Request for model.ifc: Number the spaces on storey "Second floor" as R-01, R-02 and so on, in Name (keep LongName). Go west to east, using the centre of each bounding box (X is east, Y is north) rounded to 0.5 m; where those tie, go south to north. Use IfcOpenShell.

First a look at what the model holds.

```python
import ifcopenshell
import ifcopenshell.util.element
import ifcopenshell.util.placement

model = ifcopenshell.open("model.ifc")
print(model.schema)
storey = next(s for s in model.by_type("IfcBuildingStorey") if s.Name == "Second floor")
spaces = [e for e in ifcopenshell.util.element.get_decomposition(storey) if e.is_a("IfcSpace")]
for e in sorted(spaces, key=lambda e: e.id()):
    origin = ifcopenshell.util.placement.get_local_placement(e.ObjectPlacement)[:3, 3]
    print(e.id(), e.Name, e.LongName, origin.round(2) + 0.0, sep=" | ")
```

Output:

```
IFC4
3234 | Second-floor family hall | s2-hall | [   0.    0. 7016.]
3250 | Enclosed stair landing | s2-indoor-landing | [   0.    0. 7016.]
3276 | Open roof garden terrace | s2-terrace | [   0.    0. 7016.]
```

```python
import ifcopenshell
import ifcopenshell.geom
import ifcopenshell.util.element
import ifcopenshell.util.shape

model = ifcopenshell.open("model.ifc")
settings = ifcopenshell.geom.settings()
settings.set("use-world-coords", True)


def centre(element):
    shape = ifcopenshell.geom.create_shape(settings, element)
    return ifcopenshell.util.shape.get_bbox_centroid(shape.geometry)


storey = next(s for s in model.by_type("IfcBuildingStorey") if s.Name == "Second floor")
spaces = [e for e in ifcopenshell.util.element.get_decomposition(storey) if e.is_a("IfcSpace")]

# Insertion points can sit at a corner or the storey origin, so sort by the geometry (in metres).
centres = {e: centre(e) for e in spaces}
spaces.sort(key=lambda e: (round(centres[e][0] / 0.5), centres[e][1]))

for i, e in enumerate(spaces, start=1):
    number = f"R-{i:02d}"
    e.Name = number
    print(e.id(), number)

model.write("model_edited.ifc")
```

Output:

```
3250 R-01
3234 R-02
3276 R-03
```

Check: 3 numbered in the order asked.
